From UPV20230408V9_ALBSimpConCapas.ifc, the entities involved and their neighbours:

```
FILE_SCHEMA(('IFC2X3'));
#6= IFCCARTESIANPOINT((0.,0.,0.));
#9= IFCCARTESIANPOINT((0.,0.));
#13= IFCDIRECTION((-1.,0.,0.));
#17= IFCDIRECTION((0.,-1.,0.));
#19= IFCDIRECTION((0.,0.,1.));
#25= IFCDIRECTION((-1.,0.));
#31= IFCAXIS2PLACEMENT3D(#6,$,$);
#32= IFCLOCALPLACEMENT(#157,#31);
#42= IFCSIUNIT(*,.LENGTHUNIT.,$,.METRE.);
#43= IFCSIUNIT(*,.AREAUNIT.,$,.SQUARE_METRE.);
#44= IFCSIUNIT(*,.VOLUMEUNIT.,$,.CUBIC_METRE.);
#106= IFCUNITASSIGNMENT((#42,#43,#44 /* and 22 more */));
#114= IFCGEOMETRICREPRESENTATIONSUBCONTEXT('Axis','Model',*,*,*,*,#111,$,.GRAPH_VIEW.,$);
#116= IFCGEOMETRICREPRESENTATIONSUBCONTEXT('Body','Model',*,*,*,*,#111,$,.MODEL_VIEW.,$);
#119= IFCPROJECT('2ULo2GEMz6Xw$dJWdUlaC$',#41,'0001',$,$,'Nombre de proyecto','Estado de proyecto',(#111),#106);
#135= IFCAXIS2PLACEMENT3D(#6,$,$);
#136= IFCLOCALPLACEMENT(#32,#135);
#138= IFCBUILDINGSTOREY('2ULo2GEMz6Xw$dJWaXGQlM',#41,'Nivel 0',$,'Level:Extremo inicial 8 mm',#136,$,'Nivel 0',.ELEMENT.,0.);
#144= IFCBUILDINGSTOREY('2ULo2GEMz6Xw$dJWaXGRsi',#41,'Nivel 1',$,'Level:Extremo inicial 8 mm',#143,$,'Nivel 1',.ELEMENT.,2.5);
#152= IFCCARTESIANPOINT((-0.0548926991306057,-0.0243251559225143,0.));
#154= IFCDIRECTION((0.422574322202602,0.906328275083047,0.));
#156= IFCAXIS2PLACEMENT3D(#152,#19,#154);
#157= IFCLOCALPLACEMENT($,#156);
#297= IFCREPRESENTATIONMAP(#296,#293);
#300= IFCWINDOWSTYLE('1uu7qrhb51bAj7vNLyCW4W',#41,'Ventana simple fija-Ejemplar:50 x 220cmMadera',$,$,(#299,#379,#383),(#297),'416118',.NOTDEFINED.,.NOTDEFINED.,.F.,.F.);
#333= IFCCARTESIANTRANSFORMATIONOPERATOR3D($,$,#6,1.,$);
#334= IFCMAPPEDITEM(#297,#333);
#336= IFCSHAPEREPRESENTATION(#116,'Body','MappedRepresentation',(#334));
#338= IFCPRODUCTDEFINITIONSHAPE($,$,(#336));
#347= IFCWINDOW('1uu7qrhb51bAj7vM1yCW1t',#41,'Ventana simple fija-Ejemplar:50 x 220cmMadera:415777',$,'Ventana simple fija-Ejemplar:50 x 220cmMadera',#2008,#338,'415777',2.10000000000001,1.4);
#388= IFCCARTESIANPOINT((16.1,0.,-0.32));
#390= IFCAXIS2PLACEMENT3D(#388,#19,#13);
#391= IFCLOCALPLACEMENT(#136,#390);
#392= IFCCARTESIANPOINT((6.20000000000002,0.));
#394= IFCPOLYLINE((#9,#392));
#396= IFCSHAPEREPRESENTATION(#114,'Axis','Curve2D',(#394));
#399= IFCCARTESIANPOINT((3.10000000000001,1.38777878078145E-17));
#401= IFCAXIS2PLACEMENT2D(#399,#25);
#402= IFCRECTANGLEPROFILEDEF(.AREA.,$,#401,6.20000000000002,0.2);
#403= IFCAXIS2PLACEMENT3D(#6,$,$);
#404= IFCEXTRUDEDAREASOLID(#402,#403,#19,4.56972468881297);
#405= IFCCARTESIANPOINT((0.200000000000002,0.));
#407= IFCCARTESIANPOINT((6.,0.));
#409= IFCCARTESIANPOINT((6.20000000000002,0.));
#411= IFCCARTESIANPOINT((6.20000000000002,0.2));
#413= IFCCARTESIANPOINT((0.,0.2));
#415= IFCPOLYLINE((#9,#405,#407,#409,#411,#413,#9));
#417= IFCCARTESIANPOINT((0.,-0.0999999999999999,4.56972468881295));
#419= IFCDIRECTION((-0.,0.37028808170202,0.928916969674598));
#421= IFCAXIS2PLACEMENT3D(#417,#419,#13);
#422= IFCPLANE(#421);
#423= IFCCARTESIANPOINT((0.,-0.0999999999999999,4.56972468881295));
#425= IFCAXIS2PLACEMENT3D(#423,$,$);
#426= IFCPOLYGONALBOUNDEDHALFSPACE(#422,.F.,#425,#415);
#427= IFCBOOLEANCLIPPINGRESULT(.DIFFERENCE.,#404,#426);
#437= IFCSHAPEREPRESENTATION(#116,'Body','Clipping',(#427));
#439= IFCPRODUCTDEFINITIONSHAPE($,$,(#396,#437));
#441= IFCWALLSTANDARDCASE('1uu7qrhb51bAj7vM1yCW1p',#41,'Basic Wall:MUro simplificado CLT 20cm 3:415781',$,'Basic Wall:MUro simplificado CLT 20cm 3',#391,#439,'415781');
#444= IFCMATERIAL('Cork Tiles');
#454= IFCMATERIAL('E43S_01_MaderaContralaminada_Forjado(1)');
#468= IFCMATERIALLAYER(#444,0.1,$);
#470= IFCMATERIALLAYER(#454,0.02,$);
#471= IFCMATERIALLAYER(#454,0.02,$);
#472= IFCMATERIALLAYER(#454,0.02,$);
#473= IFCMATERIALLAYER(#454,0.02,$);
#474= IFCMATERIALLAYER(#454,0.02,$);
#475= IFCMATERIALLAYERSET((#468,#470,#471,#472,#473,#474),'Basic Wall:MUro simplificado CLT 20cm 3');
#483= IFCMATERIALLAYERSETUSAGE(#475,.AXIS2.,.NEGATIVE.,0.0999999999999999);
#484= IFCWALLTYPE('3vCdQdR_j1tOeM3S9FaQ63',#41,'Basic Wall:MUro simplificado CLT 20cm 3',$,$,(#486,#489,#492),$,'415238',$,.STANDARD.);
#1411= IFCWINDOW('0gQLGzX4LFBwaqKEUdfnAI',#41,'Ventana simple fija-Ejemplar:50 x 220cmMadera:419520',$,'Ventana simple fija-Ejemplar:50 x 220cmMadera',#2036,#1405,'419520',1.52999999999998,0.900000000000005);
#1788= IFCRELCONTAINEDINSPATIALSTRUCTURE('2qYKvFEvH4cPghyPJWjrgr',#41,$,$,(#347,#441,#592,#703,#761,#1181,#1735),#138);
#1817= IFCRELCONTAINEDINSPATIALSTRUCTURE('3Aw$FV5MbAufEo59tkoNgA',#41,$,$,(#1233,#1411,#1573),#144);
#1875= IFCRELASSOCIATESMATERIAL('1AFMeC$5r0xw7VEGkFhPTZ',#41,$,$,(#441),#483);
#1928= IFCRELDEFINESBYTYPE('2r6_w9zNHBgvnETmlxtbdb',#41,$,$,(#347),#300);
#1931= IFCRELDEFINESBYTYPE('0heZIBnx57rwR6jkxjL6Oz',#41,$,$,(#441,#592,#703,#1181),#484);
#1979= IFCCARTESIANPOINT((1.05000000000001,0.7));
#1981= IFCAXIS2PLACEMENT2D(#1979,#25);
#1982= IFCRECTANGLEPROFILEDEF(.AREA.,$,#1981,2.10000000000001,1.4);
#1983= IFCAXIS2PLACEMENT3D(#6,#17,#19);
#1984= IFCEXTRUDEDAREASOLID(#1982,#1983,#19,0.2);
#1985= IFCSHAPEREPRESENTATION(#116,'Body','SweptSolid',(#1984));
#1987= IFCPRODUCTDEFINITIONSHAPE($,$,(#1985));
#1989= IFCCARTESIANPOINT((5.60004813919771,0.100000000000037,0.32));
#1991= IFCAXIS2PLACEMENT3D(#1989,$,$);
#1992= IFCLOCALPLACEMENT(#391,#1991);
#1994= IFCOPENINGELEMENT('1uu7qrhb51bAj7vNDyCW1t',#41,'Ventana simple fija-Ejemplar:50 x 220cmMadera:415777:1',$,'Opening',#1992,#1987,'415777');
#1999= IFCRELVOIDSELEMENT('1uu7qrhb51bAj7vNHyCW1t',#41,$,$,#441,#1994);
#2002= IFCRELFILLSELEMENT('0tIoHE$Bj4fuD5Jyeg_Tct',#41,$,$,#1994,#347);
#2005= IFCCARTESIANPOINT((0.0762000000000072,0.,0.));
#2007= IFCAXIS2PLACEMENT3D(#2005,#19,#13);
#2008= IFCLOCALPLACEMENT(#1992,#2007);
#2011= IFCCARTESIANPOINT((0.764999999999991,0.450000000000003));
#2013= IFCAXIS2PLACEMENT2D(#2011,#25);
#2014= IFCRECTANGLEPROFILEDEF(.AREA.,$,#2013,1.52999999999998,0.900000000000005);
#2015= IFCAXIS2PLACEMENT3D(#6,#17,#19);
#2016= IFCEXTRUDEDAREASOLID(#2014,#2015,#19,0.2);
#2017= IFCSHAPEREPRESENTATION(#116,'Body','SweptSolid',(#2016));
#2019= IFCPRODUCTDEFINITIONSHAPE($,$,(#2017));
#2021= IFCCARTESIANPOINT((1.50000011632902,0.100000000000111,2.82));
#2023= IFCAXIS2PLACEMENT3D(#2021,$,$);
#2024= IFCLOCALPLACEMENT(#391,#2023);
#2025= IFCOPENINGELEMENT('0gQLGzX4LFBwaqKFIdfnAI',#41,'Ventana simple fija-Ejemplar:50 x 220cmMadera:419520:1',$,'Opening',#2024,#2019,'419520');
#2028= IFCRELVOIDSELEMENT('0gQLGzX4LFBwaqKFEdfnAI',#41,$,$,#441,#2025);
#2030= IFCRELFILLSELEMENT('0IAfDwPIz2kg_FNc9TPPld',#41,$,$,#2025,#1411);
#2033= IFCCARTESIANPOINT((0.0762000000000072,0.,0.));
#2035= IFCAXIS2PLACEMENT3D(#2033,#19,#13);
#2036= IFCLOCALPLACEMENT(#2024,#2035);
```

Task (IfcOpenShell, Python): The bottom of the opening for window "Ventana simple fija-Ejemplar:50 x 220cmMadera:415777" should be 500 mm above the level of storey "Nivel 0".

```python
import numpy as np
import ifcopenshell
import ifcopenshell.api.geometry
import ifcopenshell.geom
import ifcopenshell.util.element
import ifcopenshell.util.placement
import ifcopenshell.util.shape
import ifcopenshell.util.unit

model = ifcopenshell.open("UPV20230408V9_ALBSimpConCapas.ifc")
unit_scale = ifcopenshell.util.unit.calculate_unit_scale(model)

window = model.by_guid("1uu7qrhb51bAj7vM1yCW1t")
opening = window.FillsVoids[0].RelatingOpeningElement
storey = ifcopenshell.util.element.get_container(window, ifc_class="IfcBuildingStorey")
level = ifcopenshell.util.placement.get_local_placement(storey.ObjectPlacement)[2, 3]

# The opening's origin need not be at the sill, so measure its lowest point.
shape = ifcopenshell.geom.create_shape(ifcopenshell.geom.settings(), opening)
bottom = ifcopenshell.util.shape.get_shape_bottom_elevation(shape, shape.geometry) / unit_scale
dz = level + 0.5 - bottom

shift = np.array([0.0, 0.0, dz])
# The window is placed relative to its opening, so it follows when the opening moves.
matrix = ifcopenshell.util.placement.get_local_placement(opening.ObjectPlacement)
matrix[:3, 3] += shift
ifcopenshell.api.geometry.edit_object_placement(
    model, product=opening, matrix=matrix, is_si=False, should_transform_children=True
)

print(f"moved by {dz * unit_scale:+.3f} m")

model.write("UPV20230408V9_ALBSimpConCapas_updated.ifc")
```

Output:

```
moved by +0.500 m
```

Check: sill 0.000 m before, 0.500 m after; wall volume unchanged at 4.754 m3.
